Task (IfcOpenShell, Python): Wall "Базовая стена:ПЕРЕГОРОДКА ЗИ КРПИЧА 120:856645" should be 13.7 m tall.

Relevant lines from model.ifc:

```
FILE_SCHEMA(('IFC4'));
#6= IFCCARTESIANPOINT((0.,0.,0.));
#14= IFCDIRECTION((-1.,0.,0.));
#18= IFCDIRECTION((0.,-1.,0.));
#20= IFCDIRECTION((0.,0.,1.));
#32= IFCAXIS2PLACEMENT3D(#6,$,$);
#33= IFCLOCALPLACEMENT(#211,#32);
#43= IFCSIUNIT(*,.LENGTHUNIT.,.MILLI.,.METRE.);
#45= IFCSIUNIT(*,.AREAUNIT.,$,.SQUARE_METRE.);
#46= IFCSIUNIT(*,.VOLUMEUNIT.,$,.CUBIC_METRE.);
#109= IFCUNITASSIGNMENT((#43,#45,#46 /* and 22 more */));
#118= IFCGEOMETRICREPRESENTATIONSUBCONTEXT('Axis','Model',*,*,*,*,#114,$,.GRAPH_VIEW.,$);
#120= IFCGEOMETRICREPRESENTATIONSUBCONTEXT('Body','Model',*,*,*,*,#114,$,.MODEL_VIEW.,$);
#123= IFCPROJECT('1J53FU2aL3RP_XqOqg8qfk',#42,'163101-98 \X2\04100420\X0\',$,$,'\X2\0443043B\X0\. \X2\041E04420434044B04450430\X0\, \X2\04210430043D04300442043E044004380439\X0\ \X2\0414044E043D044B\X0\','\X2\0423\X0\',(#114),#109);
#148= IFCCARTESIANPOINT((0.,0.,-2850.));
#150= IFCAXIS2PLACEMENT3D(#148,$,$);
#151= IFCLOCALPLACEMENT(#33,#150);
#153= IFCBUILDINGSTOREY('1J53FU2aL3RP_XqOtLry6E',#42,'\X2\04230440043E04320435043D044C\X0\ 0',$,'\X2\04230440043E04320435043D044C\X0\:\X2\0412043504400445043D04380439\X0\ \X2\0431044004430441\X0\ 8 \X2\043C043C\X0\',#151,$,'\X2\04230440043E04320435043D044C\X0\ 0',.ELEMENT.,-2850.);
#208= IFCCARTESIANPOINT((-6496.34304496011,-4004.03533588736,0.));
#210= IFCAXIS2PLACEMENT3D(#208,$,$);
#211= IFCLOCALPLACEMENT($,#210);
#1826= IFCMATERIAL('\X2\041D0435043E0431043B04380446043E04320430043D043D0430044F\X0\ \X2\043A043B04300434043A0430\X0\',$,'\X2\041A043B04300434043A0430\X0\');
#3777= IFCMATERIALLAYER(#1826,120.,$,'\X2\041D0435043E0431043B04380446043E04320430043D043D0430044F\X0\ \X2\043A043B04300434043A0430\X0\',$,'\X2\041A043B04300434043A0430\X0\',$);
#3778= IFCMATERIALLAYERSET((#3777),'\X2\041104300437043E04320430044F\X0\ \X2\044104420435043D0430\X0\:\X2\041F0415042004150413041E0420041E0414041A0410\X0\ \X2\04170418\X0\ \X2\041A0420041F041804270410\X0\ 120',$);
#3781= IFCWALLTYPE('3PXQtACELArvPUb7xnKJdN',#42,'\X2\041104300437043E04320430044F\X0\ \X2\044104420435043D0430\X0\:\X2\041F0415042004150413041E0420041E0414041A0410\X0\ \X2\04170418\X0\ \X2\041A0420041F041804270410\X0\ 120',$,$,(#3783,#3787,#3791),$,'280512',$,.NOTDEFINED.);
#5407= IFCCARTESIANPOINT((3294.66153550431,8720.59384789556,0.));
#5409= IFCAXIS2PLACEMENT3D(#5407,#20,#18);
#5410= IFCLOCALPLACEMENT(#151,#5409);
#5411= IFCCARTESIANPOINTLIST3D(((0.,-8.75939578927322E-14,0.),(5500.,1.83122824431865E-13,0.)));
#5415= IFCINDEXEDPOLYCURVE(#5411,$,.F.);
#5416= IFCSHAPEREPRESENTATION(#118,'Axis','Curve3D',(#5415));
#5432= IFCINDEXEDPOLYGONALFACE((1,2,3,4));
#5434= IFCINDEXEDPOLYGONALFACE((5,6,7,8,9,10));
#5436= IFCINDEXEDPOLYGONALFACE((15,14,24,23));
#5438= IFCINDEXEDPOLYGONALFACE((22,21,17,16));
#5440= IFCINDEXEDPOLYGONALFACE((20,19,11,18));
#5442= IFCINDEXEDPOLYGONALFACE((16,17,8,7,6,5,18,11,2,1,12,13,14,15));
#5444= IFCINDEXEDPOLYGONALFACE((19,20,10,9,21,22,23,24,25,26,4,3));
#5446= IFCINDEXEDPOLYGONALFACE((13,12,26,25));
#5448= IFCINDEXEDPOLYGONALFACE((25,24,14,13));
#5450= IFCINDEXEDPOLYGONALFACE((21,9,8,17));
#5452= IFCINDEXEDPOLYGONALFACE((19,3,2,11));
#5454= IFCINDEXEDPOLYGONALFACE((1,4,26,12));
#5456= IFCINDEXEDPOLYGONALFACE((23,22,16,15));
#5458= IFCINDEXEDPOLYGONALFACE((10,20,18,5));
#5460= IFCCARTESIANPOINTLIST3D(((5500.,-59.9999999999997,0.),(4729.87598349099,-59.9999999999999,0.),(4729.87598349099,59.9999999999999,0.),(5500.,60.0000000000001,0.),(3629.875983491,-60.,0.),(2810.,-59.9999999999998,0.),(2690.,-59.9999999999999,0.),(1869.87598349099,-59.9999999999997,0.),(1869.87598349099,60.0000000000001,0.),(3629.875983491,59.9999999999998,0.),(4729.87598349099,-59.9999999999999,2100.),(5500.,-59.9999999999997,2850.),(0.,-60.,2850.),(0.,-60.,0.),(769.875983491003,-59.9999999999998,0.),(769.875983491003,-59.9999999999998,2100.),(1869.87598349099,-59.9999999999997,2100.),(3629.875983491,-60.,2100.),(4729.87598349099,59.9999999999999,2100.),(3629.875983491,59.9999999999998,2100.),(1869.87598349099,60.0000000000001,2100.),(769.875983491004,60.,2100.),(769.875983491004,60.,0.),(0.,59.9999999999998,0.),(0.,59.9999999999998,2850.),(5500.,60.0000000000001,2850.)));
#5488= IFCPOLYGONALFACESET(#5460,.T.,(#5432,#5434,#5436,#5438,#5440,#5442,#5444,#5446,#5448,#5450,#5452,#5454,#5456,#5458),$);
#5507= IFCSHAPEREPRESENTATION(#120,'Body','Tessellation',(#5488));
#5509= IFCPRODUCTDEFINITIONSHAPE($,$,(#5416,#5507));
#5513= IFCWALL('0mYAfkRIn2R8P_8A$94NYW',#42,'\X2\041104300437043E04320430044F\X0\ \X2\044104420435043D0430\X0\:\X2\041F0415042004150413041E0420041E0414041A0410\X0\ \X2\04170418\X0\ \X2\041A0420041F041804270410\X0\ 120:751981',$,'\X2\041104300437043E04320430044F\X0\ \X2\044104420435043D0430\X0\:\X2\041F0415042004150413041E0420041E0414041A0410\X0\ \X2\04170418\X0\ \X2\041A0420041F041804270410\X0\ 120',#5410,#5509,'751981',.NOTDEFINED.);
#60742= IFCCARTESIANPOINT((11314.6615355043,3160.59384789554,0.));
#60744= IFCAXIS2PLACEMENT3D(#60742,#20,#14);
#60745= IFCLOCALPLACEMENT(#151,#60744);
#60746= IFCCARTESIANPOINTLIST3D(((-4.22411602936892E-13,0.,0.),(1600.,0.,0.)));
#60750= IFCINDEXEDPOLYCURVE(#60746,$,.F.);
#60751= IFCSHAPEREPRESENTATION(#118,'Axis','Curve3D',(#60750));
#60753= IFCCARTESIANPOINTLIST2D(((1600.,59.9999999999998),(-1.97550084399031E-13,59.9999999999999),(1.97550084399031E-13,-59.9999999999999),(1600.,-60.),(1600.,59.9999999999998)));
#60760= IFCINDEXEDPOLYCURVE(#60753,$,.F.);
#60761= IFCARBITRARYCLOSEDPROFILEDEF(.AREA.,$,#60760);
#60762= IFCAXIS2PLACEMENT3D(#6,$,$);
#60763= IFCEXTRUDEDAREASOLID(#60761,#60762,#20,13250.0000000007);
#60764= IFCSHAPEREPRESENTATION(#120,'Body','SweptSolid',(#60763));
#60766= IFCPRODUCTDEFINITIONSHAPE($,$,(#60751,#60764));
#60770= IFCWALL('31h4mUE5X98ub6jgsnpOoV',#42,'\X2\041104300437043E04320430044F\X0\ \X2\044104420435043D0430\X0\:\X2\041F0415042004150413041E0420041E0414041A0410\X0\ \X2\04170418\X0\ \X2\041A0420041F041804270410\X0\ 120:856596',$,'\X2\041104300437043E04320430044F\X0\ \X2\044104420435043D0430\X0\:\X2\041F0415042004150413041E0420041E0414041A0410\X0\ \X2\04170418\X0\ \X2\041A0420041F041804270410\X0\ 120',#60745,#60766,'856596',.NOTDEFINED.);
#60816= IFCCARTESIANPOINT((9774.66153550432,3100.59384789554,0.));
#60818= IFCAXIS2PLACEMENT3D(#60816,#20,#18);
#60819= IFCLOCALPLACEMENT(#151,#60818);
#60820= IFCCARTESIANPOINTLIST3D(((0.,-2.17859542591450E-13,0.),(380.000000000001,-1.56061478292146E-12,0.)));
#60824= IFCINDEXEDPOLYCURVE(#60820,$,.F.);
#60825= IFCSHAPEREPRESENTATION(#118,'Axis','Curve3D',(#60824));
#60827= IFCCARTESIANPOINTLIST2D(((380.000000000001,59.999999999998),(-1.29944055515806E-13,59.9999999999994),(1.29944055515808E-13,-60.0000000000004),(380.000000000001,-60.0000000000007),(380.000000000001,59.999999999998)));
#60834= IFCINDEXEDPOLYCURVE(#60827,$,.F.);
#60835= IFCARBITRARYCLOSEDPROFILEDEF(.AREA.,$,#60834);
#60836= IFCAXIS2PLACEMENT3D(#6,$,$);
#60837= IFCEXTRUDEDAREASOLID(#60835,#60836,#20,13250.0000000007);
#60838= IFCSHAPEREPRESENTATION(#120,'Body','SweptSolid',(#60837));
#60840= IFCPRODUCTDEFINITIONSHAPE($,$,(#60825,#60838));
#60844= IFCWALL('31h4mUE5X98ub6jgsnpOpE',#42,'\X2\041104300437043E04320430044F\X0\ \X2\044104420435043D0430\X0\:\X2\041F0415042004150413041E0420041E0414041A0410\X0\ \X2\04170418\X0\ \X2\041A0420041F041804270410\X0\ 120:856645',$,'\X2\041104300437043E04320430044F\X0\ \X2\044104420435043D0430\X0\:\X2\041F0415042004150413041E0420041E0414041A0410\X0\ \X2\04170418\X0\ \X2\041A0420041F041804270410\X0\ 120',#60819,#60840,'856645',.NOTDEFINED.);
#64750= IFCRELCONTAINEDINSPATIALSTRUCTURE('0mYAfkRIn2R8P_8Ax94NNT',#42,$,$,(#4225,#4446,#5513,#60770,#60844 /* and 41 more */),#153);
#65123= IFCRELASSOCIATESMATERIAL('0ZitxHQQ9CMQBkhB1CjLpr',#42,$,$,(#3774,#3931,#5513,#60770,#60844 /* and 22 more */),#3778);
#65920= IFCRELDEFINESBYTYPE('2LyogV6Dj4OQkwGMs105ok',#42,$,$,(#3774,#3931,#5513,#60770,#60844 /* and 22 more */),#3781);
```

```python
import ifcopenshell
import ifcopenshell.geom
import ifcopenshell.util.representation
import ifcopenshell.util.shape

model = ifcopenshell.open("model.ifc")
settings = ifcopenshell.geom.settings()


def volume(element):
    """Net volume in cubic metres, openings subtracted."""
    shape = ifcopenshell.geom.create_shape(settings, element)
    return ifcopenshell.util.shape.get_volume(shape.geometry)


wall = model.by_guid("31h4mUE5X98ub6jgsnpOpE")
before = volume(wall)

body = ifcopenshell.util.representation.get_representation(wall, "Model", "Body")
solid = body.Items[0]
old_height = solid.Depth
solid.Depth = 13700.0
after = volume(wall)

print(f"height {old_height:g} -> {solid.Depth:g}, volume {before:.3f} -> {after:.3f} m3")

model.write("model_updated.ifc")
```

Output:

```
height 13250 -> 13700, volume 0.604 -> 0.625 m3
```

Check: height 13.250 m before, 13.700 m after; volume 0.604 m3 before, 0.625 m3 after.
